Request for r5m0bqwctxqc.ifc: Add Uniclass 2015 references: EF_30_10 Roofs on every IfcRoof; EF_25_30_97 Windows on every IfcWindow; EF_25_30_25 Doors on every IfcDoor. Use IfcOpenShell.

First a look at what the model holds.

```python
import ifcopenshell

model = ifcopenshell.open("r5m0bqwctxqc.ifc")
print(model.schema)
print("classifications:", [c.Name for c in model.by_type("IfcClassification")])
for ifc_class in ("IfcDoor", "IfcRoof", "IfcStair", "IfcWall", "IfcWindow"):
    print(ifc_class, len(model.by_type(ifc_class)))
```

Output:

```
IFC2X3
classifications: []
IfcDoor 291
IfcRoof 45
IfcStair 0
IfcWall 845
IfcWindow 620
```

```python
import ifcopenshell
import ifcopenshell.api.classification

model = ifcopenshell.open("r5m0bqwctxqc.ifc")

# IFC2X3 requires Source and Edition and has no link from the project to the system.
system = model.create_entity("IfcClassification", Source="NBS", Edition="2015", Name="Uniclass 2015")

codes = {
    "IfcRoof": ("EF_30_10", "Roofs"),
    "IfcWindow": ("EF_25_30_97", "Windows"),
    "IfcDoor": ("EF_25_30_25", "Doors"),
}
for ifc_class, (code, name) in codes.items():
    products = model.by_type(ifc_class)
    ifcopenshell.api.classification.add_reference(
        model, products=products, classification=system, identification=code, name=name
    )
    print(code, len(products))

model.write("r5m0bqwctxqc_v2.ifc")
```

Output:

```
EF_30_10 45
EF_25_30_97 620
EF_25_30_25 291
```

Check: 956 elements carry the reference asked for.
